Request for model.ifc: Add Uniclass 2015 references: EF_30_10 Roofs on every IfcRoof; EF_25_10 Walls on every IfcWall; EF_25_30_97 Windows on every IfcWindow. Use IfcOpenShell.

First a look at what the model holds.

```python
import ifcopenshell

model = ifcopenshell.open("model.ifc")
print(model.schema)
print("classifications:", [c.Name for c in model.by_type("IfcClassification")])
for ifc_class in ("IfcDoor", "IfcRoof", "IfcStair", "IfcWall", "IfcWindow"):
    print(ifc_class, len(model.by_type(ifc_class)))
```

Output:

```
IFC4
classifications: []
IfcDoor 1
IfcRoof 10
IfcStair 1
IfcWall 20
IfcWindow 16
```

```python
import ifcopenshell
import ifcopenshell.api.classification

model = ifcopenshell.open("model.ifc")

system = ifcopenshell.api.classification.add_classification(model, classification="Uniclass 2015")

codes = {
    "IfcRoof": ("EF_30_10", "Roofs"),
    "IfcWall": ("EF_25_10", "Walls"),
    "IfcWindow": ("EF_25_30_97", "Windows"),
}
for ifc_class, (code, name) in codes.items():
    products = model.by_type(ifc_class)
    ifcopenshell.api.classification.add_reference(
        model, products=products, classification=system, identification=code, name=name
    )
    print(code, len(products))

model.write("model-out.ifc")
```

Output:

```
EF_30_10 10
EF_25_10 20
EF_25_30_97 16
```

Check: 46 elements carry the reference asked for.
